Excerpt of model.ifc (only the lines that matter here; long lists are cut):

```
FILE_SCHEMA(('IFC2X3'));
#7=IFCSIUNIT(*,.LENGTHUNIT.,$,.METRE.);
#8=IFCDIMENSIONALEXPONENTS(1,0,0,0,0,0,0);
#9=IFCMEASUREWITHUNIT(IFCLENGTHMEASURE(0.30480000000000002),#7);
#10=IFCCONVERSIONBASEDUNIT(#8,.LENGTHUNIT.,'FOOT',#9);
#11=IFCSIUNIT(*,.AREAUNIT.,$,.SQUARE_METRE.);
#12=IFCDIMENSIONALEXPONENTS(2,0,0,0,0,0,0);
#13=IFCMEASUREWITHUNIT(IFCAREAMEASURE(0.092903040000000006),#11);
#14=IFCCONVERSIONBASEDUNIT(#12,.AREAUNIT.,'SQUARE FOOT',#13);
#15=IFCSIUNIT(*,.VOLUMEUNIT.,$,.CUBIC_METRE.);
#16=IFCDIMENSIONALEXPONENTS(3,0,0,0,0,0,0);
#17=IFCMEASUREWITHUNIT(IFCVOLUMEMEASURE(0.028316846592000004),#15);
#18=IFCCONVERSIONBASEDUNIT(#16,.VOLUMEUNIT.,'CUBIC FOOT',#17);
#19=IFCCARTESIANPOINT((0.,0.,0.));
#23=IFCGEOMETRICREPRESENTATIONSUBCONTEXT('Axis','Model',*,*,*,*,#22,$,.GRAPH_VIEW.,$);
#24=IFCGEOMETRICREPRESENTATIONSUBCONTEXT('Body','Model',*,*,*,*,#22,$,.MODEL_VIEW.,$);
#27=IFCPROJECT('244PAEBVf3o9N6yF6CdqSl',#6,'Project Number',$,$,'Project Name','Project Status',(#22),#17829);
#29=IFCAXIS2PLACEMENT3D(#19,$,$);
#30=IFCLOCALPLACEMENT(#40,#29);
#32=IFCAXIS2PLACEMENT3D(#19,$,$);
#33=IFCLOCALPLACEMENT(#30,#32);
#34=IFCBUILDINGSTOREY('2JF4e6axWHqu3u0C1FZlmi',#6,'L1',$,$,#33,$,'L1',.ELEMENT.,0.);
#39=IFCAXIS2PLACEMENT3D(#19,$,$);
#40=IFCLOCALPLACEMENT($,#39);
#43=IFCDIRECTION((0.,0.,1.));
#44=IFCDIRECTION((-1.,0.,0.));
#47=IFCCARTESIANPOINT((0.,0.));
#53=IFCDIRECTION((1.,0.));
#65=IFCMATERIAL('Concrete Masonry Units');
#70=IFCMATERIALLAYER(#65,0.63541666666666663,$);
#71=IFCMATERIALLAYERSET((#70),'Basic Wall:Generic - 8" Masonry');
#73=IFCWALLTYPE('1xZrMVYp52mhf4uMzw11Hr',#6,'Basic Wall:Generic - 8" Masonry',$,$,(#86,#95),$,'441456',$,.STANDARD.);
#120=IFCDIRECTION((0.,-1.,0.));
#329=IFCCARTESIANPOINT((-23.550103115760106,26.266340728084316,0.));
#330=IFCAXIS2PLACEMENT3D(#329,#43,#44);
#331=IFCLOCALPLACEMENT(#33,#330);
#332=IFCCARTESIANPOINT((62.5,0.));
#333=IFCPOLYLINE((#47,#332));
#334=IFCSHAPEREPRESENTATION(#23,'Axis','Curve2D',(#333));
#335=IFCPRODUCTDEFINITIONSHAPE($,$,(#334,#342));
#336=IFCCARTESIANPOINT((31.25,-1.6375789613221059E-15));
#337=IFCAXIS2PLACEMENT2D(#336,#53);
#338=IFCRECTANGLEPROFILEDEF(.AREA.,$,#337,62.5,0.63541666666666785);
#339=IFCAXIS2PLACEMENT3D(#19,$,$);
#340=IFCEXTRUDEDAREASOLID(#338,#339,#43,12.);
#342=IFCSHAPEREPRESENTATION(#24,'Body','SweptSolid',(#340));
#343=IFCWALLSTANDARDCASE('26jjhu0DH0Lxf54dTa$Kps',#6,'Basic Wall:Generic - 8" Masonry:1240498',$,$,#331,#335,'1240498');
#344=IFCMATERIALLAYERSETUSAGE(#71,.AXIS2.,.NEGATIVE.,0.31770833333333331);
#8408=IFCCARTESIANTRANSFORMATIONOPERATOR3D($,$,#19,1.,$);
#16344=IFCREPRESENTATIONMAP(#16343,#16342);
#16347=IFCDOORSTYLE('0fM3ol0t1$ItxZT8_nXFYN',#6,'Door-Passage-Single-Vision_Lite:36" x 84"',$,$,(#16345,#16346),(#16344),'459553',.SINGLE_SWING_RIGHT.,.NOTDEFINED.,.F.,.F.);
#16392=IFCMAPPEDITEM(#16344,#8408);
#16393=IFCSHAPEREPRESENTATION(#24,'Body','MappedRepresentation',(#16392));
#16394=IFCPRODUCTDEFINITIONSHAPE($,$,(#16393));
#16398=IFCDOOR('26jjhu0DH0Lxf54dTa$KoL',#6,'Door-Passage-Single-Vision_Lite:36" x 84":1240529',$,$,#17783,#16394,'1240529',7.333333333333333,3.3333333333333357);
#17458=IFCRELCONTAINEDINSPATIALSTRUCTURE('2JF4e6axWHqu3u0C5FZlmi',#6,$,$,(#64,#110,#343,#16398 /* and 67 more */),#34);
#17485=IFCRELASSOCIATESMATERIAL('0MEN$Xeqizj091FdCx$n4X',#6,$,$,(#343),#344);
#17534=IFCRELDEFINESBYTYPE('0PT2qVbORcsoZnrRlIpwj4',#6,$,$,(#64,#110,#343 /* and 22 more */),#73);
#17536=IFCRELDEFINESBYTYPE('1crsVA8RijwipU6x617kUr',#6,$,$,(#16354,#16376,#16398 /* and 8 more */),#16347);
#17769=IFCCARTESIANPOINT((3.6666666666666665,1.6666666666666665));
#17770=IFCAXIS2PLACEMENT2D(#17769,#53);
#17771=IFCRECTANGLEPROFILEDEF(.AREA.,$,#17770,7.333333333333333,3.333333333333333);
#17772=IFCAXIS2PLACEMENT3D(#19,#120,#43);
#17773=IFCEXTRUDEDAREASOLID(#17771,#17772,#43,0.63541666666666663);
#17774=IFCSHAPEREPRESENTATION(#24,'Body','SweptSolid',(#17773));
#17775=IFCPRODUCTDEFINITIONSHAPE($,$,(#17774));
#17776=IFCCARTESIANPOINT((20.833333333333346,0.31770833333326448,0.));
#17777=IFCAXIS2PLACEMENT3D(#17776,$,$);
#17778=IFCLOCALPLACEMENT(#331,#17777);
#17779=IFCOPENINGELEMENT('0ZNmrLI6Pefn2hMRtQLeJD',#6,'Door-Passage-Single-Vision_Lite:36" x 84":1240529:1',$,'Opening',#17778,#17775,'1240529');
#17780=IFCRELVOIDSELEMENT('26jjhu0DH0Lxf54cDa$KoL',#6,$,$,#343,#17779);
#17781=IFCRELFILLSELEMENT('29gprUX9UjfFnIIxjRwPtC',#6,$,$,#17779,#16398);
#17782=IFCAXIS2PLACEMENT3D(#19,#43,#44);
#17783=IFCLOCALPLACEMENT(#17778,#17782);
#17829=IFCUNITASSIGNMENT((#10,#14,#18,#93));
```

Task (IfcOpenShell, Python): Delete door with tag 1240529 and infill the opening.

```python
import ifcopenshell
import ifcopenshell.api.feature
import ifcopenshell.api.root
import ifcopenshell.geom
import ifcopenshell.util.shape

model = ifcopenshell.open("model.ifc")
settings = ifcopenshell.geom.settings()


def volume(element):
    """Net volume in cubic metres, openings subtracted."""
    shape = ifcopenshell.geom.create_shape(settings, element)
    return ifcopenshell.util.shape.get_volume(shape.geometry)


door = model.by_guid("26jjhu0DH0Lxf54dTa$KoL")
opening = door.FillsVoids[0].RelatingOpeningElement
wall = opening.VoidsElements[0].RelatingBuildingElement
before = volume(wall)

ifcopenshell.api.root.remove_product(model, product=door)
ifcopenshell.api.feature.remove_feature(model, feature=opening)

after = volume(wall)

print(f"wall volume {before:.3f} -> {after:.3f} m3")

model.write("model_rev.ifc")
```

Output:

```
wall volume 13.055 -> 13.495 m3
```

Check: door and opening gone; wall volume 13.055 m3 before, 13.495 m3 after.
